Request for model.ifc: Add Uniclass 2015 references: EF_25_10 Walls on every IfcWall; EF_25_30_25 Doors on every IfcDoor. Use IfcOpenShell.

First a look at what the model holds.

```python
import ifcopenshell

model = ifcopenshell.open("model.ifc")
print(model.schema)
print("classifications:", [c.Name for c in model.by_type("IfcClassification")])
for ifc_class in ("IfcDoor", "IfcRoof", "IfcStair", "IfcWall", "IfcWindow"):
    print(ifc_class, len(model.by_type(ifc_class)))
```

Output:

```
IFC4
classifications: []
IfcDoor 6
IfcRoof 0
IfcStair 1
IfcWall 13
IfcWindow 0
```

```python
import ifcopenshell
import ifcopenshell.api.classification

model = ifcopenshell.open("model.ifc")

system = ifcopenshell.api.classification.add_classification(model, classification="Uniclass 2015")

codes = {
    "IfcWall": ("EF_25_10", "Walls"),
    "IfcDoor": ("EF_25_30_25", "Doors"),
}
for ifc_class, (code, name) in codes.items():
    products = model.by_type(ifc_class)
    ifcopenshell.api.classification.add_reference(
        model, products=products, classification=system, identification=code, name=name
    )
    print(code, len(products))

model.write("model_updated.ifc")
```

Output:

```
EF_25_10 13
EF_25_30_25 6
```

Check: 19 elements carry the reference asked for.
